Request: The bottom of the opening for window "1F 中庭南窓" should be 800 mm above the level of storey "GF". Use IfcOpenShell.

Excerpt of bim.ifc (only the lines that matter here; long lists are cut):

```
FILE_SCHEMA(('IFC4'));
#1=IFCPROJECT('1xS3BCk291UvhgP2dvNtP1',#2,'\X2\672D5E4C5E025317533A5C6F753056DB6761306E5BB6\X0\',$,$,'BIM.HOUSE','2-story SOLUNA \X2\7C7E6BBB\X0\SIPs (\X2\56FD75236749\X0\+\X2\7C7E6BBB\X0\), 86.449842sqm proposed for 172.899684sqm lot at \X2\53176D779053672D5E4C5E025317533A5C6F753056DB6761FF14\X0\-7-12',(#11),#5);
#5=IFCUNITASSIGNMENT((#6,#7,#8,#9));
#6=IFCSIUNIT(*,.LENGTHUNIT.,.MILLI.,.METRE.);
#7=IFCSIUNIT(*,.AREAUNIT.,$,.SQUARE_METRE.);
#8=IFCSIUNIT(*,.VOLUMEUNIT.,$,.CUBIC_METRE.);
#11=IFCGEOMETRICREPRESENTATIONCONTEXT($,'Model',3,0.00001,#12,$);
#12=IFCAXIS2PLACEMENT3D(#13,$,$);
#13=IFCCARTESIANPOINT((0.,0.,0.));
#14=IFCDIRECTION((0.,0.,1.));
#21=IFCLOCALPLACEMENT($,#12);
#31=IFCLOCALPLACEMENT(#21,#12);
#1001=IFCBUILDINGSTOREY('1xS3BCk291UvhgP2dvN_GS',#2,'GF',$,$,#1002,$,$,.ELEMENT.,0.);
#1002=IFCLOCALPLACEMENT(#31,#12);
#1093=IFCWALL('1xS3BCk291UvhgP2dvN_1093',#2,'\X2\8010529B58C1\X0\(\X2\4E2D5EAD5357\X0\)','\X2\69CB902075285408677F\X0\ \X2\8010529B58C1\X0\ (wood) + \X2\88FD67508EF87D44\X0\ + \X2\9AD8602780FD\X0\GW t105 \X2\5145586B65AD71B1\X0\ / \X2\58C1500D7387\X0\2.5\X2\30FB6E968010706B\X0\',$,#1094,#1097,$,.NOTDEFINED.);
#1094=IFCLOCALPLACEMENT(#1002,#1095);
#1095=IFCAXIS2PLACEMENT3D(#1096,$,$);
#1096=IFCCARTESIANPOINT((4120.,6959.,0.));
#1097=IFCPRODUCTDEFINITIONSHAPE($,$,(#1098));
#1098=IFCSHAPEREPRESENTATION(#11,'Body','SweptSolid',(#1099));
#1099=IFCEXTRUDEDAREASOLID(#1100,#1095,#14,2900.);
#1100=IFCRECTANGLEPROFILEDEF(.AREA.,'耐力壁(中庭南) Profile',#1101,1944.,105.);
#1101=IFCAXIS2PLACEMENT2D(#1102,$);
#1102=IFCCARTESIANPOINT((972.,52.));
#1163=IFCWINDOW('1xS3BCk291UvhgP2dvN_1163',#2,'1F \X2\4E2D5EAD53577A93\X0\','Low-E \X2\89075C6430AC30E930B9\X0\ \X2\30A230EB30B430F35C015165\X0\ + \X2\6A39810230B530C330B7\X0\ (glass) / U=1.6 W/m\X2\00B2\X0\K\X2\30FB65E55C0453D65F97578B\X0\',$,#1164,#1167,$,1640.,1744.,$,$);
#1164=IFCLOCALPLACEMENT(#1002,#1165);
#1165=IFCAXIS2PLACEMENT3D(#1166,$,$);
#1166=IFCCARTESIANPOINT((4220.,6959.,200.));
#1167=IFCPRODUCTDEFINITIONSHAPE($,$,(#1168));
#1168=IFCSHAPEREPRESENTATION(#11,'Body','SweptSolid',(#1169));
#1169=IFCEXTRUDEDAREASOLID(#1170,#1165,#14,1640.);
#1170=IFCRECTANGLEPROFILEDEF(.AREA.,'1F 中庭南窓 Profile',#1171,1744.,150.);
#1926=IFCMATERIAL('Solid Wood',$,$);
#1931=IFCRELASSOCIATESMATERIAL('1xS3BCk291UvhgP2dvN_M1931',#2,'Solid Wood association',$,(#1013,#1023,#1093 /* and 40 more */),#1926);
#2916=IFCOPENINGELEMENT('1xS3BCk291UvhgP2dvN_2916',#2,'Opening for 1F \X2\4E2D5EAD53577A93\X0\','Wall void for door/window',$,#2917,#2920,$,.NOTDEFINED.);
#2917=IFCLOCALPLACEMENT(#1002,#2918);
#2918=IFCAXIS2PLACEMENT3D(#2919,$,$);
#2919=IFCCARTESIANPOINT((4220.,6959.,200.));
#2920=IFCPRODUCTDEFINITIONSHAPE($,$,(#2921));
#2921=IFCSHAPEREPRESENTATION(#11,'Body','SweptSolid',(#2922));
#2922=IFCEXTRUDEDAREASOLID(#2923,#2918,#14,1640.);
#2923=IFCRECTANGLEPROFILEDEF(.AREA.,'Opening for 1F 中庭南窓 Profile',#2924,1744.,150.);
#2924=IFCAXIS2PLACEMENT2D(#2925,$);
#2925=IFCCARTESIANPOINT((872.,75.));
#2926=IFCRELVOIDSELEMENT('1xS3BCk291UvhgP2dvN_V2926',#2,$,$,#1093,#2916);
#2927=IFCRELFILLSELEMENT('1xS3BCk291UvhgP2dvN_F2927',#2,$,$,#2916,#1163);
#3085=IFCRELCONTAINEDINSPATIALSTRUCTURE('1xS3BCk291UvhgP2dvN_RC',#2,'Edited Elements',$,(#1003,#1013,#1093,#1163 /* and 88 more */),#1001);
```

```python
import numpy as np
import ifcopenshell
import ifcopenshell.api.geometry
import ifcopenshell.geom
import ifcopenshell.util.element
import ifcopenshell.util.placement
import ifcopenshell.util.shape
import ifcopenshell.util.unit

model = ifcopenshell.open("bim.ifc")
unit_scale = ifcopenshell.util.unit.calculate_unit_scale(model)

window = model.by_guid("1xS3BCk291UvhgP2dvN_1163")
opening = window.FillsVoids[0].RelatingOpeningElement
storey = ifcopenshell.util.element.get_container(window, ifc_class="IfcBuildingStorey")
level = ifcopenshell.util.placement.get_local_placement(storey.ObjectPlacement)[2, 3]

# The opening's origin need not be at the sill, so measure its lowest point.
shape = ifcopenshell.geom.create_shape(ifcopenshell.geom.settings(), opening)
bottom = ifcopenshell.util.shape.get_shape_bottom_elevation(shape, shape.geometry) / unit_scale
dz = level + 0.8 / unit_scale - bottom

shift = np.array([0.0, 0.0, dz])
# The window is not placed relative to its opening, so move both.
for product in (opening, window):
    matrix = ifcopenshell.util.placement.get_local_placement(product.ObjectPlacement)
    matrix[:3, 3] += shift
    ifcopenshell.api.geometry.edit_object_placement(model, product=product, matrix=matrix, is_si=False)

print(f"moved by {dz * unit_scale:+.3f} m")

model.write("bim-out.ifc")
```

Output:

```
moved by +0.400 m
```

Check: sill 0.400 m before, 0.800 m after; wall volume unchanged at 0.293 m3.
